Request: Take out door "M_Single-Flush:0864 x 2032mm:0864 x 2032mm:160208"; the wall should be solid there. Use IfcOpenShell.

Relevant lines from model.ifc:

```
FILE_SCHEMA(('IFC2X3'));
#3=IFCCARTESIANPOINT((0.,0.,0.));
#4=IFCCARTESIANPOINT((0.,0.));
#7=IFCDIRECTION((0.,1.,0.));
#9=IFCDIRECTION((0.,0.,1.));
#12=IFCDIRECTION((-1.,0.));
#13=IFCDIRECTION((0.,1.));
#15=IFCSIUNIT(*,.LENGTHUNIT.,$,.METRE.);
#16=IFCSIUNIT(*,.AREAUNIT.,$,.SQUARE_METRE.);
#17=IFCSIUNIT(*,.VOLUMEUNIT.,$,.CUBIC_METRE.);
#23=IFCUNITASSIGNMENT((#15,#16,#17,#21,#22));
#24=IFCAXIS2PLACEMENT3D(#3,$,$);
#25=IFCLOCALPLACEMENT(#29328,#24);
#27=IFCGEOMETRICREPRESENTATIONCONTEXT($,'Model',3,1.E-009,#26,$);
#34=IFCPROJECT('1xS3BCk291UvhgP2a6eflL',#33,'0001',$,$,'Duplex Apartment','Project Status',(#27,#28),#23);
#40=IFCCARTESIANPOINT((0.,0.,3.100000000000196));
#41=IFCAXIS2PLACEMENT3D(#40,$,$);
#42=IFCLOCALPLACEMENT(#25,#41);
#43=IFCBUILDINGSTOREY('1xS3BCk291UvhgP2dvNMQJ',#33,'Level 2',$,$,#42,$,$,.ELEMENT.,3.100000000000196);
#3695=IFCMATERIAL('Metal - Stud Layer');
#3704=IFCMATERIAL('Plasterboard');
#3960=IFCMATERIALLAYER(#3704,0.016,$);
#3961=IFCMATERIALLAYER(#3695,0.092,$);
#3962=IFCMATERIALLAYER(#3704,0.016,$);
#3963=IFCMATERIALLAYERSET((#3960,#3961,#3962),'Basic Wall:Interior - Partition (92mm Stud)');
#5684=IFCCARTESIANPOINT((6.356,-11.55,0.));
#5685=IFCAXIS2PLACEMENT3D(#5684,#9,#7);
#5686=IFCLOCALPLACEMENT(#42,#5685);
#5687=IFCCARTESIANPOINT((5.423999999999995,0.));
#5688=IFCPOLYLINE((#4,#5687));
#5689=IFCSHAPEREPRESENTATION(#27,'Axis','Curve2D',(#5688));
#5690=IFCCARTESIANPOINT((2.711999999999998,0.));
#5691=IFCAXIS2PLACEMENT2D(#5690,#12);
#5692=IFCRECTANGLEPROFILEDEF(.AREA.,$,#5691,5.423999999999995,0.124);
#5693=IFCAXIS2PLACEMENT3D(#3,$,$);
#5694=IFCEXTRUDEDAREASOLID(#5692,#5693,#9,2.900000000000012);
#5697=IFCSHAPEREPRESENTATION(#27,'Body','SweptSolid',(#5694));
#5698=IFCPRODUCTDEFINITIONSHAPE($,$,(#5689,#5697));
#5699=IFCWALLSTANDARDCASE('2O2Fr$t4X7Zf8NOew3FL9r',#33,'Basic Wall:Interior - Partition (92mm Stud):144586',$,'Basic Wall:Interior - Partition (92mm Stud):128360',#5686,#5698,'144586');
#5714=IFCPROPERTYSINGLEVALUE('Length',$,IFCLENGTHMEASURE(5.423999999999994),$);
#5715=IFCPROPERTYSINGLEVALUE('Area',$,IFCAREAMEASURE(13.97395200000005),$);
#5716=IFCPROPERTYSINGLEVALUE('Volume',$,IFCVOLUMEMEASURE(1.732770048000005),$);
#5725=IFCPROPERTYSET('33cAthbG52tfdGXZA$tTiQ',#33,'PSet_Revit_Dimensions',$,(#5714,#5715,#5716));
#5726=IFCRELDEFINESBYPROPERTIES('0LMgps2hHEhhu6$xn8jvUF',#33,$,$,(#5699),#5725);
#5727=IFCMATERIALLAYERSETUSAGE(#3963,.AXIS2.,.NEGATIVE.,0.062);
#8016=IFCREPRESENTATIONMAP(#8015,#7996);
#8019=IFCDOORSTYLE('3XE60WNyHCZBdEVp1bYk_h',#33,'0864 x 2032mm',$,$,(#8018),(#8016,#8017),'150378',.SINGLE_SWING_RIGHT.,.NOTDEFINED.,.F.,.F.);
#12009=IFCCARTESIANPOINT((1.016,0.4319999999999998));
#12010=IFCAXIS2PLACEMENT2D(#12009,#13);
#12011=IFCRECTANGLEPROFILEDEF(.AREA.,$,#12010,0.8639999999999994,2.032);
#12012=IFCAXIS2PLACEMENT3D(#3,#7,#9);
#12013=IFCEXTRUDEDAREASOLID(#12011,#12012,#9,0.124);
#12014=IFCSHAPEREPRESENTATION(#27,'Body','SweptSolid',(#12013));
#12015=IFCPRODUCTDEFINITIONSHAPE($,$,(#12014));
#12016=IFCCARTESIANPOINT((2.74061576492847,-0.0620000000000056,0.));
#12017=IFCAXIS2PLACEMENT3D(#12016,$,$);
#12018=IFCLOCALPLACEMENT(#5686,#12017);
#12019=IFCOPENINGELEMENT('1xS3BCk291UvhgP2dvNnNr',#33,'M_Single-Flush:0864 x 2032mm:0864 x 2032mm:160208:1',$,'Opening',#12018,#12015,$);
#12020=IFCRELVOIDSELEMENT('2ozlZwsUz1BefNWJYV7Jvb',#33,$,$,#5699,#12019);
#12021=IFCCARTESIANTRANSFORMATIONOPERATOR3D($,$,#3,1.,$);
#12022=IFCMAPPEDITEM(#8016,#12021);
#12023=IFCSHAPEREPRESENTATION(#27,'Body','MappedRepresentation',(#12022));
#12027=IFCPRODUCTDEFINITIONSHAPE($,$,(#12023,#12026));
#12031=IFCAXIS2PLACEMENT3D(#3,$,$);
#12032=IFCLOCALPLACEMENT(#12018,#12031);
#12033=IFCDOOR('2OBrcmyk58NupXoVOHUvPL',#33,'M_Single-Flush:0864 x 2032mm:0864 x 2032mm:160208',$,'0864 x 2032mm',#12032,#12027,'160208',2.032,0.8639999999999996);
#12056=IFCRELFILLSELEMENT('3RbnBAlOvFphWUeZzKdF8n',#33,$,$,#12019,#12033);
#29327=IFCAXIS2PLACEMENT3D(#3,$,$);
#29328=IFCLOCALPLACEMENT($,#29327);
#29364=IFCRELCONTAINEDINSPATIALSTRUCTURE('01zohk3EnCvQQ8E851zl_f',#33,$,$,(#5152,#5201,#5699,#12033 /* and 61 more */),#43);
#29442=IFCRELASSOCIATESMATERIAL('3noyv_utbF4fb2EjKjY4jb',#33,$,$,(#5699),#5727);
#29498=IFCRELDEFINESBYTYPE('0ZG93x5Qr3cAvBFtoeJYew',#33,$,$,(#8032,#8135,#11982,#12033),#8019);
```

```python
import ifcopenshell
import ifcopenshell.api.feature
import ifcopenshell.api.pset
import ifcopenshell.api.root
import ifcopenshell.geom
import ifcopenshell.util.element
import ifcopenshell.util.shape
import ifcopenshell.util.unit

model = ifcopenshell.open("model.ifc")
area_scale = ifcopenshell.util.unit.calculate_unit_scale(model, "AREAUNIT")
volume_scale = ifcopenshell.util.unit.calculate_unit_scale(model, "VOLUMEUNIT")
settings = ifcopenshell.geom.settings()


def volume(element):
    """Net volume in cubic metres, openings subtracted."""
    shape = ifcopenshell.geom.create_shape(settings, element)
    return ifcopenshell.util.shape.get_volume(shape.geometry)


door = model.by_guid("2OBrcmyk58NupXoVOHUvPL")
opening = door.FillsVoids[0].RelatingOpeningElement
wall = opening.VoidsElements[0].RelatingBuildingElement
before = volume(wall)

ifcopenshell.api.root.remove_product(model, product=door)
ifcopenshell.api.feature.remove_feature(model, feature=opening)

after = volume(wall)
thickness = 0.124  # wall thickness in metres

# Update the wall's stored quantities.
pset = model.by_id(ifcopenshell.util.element.get_pset(wall, "PSet_Revit_Dimensions", should_inherit=False)["id"])
ifcopenshell.api.pset.edit_pset(model, pset=pset, properties={
    "Area": model.create_entity("IfcAreaMeasure", after / thickness / area_scale),
    "Volume": model.create_entity("IfcVolumeMeasure", after / volume_scale),
})

print(f"wall volume {before:.3f} -> {after:.3f} m3")

model.write("model-out.ifc")
```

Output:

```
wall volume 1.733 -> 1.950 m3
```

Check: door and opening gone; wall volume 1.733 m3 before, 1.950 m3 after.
